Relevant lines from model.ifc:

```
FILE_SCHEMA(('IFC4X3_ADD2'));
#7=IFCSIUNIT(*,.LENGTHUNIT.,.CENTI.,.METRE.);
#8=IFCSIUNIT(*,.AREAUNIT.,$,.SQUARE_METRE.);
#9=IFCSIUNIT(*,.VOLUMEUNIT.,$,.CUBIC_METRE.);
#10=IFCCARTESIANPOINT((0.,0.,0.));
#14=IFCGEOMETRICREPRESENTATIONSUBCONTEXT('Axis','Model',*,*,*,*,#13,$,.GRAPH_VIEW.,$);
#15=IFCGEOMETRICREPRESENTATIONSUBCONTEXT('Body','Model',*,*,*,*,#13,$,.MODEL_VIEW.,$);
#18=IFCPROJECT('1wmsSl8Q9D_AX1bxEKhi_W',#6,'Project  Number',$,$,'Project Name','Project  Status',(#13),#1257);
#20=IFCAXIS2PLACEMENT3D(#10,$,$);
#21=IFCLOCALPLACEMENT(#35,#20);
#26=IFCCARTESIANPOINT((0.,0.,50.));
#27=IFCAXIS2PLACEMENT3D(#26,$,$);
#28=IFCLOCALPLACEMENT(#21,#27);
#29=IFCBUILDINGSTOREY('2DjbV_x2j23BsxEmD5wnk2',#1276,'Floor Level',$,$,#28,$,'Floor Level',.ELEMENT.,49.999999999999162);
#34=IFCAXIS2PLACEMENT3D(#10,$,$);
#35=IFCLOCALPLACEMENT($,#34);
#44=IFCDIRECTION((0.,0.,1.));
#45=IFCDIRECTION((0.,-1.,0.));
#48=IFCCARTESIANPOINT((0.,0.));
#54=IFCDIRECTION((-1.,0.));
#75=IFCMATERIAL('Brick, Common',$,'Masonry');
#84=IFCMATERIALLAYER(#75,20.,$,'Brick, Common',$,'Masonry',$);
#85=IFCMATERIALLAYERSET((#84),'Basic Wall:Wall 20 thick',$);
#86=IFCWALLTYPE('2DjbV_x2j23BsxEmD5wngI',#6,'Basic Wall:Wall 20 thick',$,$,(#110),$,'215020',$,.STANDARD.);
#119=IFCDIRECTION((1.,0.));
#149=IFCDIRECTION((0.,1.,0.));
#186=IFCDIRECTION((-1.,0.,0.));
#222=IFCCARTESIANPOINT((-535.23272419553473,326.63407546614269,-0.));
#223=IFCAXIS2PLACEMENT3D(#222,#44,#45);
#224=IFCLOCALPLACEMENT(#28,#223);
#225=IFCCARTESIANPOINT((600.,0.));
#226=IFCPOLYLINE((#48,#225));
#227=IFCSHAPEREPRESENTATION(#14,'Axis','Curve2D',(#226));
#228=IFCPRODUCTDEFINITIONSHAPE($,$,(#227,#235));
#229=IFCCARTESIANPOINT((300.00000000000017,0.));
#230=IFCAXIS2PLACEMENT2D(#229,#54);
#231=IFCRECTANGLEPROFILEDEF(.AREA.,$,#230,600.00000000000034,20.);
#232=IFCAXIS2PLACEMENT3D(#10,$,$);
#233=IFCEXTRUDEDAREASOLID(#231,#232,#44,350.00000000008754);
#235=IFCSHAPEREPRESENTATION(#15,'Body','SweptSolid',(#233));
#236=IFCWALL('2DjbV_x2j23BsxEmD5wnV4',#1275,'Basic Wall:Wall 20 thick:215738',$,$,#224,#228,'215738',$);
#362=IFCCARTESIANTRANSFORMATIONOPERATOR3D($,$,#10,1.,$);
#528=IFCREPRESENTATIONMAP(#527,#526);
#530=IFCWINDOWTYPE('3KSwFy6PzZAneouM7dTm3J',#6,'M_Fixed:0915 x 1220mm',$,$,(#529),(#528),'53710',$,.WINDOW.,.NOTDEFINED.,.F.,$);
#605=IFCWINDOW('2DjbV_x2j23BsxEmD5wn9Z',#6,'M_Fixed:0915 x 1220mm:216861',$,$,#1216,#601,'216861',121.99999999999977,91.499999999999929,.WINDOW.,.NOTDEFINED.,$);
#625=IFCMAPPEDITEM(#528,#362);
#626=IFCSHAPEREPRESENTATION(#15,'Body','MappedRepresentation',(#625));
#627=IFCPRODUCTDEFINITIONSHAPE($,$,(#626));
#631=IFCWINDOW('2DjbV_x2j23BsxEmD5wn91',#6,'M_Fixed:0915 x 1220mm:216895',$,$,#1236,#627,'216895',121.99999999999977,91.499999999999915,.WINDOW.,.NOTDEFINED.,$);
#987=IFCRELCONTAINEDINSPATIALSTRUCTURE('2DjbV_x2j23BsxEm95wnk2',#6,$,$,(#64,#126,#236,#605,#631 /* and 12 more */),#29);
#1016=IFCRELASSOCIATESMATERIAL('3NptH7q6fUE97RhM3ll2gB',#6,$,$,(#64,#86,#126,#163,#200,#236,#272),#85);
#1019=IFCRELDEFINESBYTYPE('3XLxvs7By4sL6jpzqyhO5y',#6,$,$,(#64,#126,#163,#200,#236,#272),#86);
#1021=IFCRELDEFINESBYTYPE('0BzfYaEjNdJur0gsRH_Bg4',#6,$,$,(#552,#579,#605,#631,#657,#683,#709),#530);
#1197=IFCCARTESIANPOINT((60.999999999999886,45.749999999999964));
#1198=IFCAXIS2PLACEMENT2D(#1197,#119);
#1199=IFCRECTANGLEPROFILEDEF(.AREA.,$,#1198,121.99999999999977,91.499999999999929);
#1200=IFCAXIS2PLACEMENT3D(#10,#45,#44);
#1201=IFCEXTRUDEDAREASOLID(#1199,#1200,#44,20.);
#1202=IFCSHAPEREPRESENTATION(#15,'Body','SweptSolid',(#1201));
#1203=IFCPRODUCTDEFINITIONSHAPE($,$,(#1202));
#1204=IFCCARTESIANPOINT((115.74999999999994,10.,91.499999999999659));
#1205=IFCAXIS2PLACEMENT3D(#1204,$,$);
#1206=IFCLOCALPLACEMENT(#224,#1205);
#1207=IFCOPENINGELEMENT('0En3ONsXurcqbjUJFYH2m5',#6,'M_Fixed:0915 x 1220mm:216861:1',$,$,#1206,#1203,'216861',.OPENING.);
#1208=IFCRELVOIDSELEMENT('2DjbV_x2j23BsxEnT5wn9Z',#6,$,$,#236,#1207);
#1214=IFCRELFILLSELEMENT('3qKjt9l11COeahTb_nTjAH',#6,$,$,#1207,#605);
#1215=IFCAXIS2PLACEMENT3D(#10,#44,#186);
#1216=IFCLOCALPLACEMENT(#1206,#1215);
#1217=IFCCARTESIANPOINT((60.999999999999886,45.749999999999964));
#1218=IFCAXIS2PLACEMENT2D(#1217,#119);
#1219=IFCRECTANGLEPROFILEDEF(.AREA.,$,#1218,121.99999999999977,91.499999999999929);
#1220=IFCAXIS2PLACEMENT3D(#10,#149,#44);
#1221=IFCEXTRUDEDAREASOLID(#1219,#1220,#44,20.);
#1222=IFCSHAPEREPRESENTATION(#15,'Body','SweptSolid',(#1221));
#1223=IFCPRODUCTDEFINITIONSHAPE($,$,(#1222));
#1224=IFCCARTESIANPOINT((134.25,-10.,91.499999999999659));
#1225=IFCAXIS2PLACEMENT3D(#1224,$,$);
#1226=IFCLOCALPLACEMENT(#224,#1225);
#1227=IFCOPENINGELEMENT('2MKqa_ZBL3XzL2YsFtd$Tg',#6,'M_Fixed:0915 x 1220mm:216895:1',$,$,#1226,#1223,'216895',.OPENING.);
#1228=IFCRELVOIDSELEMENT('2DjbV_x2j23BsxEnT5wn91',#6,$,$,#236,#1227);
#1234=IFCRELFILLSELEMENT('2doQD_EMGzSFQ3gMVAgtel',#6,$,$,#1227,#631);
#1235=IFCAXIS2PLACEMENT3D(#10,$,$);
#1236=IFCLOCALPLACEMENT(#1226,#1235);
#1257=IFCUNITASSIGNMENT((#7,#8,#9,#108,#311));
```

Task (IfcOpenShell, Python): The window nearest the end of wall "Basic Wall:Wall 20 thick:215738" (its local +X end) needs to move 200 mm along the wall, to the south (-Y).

```python
import ifcopenshell
import ifcopenshell.api.geometry
import ifcopenshell.util.placement
import ifcopenshell.util.unit

model = ifcopenshell.open("model.ifc")
unit_scale = ifcopenshell.util.unit.calculate_unit_scale(model)

window = model.by_id(631)
opening = window.FillsVoids[0].RelatingOpeningElement
wall = opening.VoidsElements[0].RelatingBuildingElement

wall_matrix = ifcopenshell.util.placement.get_local_placement(wall.ObjectPlacement)
shift = wall_matrix[:3, 0] * 0.2 / unit_scale
before = ifcopenshell.util.placement.get_local_placement(window.ObjectPlacement)[:3, 3].copy()

# The window is placed relative to its opening, so it follows when the opening moves.
matrix = ifcopenshell.util.placement.get_local_placement(opening.ObjectPlacement)
matrix[:3, 3] += shift
ifcopenshell.api.geometry.edit_object_placement(
    model, product=opening, matrix=matrix, is_si=False, should_transform_children=True
)

after = ifcopenshell.util.placement.get_local_placement(window.ObjectPlacement)[:3, 3]
print("window moved by", (after - before).round(3) + 0.0)

model.write("model_updated.ifc")
```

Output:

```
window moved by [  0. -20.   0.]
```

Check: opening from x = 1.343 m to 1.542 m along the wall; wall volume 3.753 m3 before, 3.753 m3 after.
